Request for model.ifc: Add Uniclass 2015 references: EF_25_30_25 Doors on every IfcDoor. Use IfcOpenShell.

First a look at what the model holds.

```python
import ifcopenshell

model = ifcopenshell.open("model.ifc")
print(model.schema)
print("classifications:", [c.Name for c in model.by_type("IfcClassification")])
for ifc_class in ("IfcDoor", "IfcRoof", "IfcStair", "IfcWall", "IfcWindow"):
    print(ifc_class, len(model.by_type(ifc_class)))
```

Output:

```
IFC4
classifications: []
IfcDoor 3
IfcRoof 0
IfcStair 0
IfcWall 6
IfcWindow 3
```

```python
import ifcopenshell
import ifcopenshell.api.classification

model = ifcopenshell.open("model.ifc")

system = ifcopenshell.api.classification.add_classification(model, classification="Uniclass 2015")

codes = {
    "IfcDoor": ("EF_25_30_25", "Doors"),
}
for ifc_class, (code, name) in codes.items():
    products = model.by_type(ifc_class)
    ifcopenshell.api.classification.add_reference(
        model, products=products, classification=system, identification=code, name=name
    )
    print(code, len(products))

model.write("model-out.ifc")
```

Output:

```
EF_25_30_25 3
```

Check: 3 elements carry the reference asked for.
